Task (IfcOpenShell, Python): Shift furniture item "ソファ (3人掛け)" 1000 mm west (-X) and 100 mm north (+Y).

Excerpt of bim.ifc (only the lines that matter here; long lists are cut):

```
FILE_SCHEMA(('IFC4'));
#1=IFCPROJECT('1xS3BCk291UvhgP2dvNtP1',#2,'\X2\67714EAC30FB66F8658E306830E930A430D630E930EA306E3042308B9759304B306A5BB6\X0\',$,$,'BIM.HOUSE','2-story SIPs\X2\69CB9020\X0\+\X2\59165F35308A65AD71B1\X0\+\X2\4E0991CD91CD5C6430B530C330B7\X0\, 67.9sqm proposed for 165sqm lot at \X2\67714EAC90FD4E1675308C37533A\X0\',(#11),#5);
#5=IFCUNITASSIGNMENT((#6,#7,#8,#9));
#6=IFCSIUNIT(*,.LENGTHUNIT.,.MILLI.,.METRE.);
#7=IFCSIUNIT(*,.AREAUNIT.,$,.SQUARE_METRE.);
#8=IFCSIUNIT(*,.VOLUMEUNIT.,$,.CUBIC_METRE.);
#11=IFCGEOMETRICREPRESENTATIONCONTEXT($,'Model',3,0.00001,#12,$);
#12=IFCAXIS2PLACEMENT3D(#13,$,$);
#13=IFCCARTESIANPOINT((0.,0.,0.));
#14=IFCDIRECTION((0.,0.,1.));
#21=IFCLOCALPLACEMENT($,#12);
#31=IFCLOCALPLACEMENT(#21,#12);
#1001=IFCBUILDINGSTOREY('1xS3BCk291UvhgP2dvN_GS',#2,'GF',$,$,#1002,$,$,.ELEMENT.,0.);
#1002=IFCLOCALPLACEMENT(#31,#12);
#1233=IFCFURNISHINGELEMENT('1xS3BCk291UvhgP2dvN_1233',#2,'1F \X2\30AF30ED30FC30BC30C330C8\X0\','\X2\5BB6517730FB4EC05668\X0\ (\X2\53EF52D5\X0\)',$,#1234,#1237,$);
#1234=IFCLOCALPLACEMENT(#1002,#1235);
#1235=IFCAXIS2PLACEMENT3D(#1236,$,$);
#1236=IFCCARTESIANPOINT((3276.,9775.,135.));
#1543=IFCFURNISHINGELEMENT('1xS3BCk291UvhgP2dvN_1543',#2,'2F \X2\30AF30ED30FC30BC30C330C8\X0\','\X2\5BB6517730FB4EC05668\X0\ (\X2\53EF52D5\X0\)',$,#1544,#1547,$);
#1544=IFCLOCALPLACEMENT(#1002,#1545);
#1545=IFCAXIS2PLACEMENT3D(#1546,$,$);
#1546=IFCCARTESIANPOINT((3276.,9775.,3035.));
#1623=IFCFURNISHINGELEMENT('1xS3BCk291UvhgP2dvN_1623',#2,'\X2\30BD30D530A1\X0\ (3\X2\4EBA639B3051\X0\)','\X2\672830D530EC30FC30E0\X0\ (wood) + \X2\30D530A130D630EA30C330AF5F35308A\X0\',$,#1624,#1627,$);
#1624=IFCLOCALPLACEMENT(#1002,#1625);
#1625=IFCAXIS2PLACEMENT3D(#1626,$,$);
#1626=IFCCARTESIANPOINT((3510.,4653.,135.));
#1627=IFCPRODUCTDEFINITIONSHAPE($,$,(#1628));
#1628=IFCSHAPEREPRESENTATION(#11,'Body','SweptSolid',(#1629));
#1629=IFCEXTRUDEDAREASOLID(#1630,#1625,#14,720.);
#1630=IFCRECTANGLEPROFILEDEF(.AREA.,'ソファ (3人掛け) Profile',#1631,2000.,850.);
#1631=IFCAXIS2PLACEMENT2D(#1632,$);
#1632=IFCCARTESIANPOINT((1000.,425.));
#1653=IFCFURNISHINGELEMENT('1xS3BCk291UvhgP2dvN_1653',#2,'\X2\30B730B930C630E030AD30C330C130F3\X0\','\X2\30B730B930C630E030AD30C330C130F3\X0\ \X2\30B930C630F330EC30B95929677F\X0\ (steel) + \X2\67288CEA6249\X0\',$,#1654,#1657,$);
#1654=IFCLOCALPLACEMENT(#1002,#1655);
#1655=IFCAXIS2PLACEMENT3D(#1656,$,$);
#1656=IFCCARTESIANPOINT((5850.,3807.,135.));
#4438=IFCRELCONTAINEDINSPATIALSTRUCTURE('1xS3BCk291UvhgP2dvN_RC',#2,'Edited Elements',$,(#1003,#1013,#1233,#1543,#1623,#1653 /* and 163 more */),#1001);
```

```python
import ifcopenshell
import ifcopenshell.api.geometry
import ifcopenshell.util.placement
import ifcopenshell.util.unit

model = ifcopenshell.open("bim.ifc")
unit_scale = ifcopenshell.util.unit.calculate_unit_scale(model)

item = model.by_guid("1xS3BCk291UvhgP2dvN_1623")
matrix = ifcopenshell.util.placement.get_local_placement(item.ObjectPlacement)
matrix[0, 3] -= 1 / unit_scale
matrix[1, 3] += 0.1 / unit_scale
ifcopenshell.api.geometry.edit_object_placement(model, product=item, matrix=matrix, is_si=False)

print(ifcopenshell.util.placement.get_local_placement(item.ObjectPlacement).round(3) + 0.0)

model.write("bim_v2.ifc")
```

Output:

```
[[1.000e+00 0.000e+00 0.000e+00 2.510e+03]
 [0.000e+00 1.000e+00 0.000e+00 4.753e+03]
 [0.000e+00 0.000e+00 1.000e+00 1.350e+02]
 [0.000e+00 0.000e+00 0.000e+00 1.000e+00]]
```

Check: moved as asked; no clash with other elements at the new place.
